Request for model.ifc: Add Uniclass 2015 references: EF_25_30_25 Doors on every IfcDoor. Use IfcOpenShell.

First a look at what the model holds.

```python
import ifcopenshell

model = ifcopenshell.open("model.ifc")
print(model.schema)
print("classifications:", [c.Name for c in model.by_type("IfcClassification")])
for ifc_class in ("IfcDoor", "IfcRoof", "IfcStair", "IfcWall", "IfcWindow"):
    print(ifc_class, len(model.by_type(ifc_class)))
```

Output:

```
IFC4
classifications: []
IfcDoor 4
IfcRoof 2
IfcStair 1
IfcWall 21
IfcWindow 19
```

```python
import ifcopenshell
import ifcopenshell.api.classification

model = ifcopenshell.open("model.ifc")

system = ifcopenshell.api.classification.add_classification(model, classification="Uniclass 2015")

codes = {
    "IfcDoor": ("EF_25_30_25", "Doors"),
}
for ifc_class, (code, name) in codes.items():
    products = model.by_type(ifc_class)
    ifcopenshell.api.classification.add_reference(
        model, products=products, classification=system, identification=code, name=name
    )
    print(code, len(products))

model.write("model_updated.ifc")
```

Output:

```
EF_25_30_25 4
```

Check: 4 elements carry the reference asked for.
